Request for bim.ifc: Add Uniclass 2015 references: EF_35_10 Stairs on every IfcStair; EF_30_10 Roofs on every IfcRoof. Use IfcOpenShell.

First a look at what the model holds.

```python
import ifcopenshell

model = ifcopenshell.open("bim.ifc")
print(model.schema)
print("classifications:", [c.Name for c in model.by_type("IfcClassification")])
for ifc_class in ("IfcDoor", "IfcRoof", "IfcStair", "IfcWall", "IfcWindow"):
    print(ifc_class, len(model.by_type(ifc_class)))
```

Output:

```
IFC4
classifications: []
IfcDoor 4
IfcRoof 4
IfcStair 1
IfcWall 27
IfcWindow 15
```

```python
import ifcopenshell
import ifcopenshell.api.classification

model = ifcopenshell.open("bim.ifc")

system = ifcopenshell.api.classification.add_classification(model, classification="Uniclass 2015")

codes = {
    "IfcStair": ("EF_35_10", "Stairs"),
    "IfcRoof": ("EF_30_10", "Roofs"),
}
for ifc_class, (code, name) in codes.items():
    products = model.by_type(ifc_class)
    ifcopenshell.api.classification.add_reference(
        model, products=products, classification=system, identification=code, name=name
    )
    print(code, len(products))

model.write("bim-out.ifc")
```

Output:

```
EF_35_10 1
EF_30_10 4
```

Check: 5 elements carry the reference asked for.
